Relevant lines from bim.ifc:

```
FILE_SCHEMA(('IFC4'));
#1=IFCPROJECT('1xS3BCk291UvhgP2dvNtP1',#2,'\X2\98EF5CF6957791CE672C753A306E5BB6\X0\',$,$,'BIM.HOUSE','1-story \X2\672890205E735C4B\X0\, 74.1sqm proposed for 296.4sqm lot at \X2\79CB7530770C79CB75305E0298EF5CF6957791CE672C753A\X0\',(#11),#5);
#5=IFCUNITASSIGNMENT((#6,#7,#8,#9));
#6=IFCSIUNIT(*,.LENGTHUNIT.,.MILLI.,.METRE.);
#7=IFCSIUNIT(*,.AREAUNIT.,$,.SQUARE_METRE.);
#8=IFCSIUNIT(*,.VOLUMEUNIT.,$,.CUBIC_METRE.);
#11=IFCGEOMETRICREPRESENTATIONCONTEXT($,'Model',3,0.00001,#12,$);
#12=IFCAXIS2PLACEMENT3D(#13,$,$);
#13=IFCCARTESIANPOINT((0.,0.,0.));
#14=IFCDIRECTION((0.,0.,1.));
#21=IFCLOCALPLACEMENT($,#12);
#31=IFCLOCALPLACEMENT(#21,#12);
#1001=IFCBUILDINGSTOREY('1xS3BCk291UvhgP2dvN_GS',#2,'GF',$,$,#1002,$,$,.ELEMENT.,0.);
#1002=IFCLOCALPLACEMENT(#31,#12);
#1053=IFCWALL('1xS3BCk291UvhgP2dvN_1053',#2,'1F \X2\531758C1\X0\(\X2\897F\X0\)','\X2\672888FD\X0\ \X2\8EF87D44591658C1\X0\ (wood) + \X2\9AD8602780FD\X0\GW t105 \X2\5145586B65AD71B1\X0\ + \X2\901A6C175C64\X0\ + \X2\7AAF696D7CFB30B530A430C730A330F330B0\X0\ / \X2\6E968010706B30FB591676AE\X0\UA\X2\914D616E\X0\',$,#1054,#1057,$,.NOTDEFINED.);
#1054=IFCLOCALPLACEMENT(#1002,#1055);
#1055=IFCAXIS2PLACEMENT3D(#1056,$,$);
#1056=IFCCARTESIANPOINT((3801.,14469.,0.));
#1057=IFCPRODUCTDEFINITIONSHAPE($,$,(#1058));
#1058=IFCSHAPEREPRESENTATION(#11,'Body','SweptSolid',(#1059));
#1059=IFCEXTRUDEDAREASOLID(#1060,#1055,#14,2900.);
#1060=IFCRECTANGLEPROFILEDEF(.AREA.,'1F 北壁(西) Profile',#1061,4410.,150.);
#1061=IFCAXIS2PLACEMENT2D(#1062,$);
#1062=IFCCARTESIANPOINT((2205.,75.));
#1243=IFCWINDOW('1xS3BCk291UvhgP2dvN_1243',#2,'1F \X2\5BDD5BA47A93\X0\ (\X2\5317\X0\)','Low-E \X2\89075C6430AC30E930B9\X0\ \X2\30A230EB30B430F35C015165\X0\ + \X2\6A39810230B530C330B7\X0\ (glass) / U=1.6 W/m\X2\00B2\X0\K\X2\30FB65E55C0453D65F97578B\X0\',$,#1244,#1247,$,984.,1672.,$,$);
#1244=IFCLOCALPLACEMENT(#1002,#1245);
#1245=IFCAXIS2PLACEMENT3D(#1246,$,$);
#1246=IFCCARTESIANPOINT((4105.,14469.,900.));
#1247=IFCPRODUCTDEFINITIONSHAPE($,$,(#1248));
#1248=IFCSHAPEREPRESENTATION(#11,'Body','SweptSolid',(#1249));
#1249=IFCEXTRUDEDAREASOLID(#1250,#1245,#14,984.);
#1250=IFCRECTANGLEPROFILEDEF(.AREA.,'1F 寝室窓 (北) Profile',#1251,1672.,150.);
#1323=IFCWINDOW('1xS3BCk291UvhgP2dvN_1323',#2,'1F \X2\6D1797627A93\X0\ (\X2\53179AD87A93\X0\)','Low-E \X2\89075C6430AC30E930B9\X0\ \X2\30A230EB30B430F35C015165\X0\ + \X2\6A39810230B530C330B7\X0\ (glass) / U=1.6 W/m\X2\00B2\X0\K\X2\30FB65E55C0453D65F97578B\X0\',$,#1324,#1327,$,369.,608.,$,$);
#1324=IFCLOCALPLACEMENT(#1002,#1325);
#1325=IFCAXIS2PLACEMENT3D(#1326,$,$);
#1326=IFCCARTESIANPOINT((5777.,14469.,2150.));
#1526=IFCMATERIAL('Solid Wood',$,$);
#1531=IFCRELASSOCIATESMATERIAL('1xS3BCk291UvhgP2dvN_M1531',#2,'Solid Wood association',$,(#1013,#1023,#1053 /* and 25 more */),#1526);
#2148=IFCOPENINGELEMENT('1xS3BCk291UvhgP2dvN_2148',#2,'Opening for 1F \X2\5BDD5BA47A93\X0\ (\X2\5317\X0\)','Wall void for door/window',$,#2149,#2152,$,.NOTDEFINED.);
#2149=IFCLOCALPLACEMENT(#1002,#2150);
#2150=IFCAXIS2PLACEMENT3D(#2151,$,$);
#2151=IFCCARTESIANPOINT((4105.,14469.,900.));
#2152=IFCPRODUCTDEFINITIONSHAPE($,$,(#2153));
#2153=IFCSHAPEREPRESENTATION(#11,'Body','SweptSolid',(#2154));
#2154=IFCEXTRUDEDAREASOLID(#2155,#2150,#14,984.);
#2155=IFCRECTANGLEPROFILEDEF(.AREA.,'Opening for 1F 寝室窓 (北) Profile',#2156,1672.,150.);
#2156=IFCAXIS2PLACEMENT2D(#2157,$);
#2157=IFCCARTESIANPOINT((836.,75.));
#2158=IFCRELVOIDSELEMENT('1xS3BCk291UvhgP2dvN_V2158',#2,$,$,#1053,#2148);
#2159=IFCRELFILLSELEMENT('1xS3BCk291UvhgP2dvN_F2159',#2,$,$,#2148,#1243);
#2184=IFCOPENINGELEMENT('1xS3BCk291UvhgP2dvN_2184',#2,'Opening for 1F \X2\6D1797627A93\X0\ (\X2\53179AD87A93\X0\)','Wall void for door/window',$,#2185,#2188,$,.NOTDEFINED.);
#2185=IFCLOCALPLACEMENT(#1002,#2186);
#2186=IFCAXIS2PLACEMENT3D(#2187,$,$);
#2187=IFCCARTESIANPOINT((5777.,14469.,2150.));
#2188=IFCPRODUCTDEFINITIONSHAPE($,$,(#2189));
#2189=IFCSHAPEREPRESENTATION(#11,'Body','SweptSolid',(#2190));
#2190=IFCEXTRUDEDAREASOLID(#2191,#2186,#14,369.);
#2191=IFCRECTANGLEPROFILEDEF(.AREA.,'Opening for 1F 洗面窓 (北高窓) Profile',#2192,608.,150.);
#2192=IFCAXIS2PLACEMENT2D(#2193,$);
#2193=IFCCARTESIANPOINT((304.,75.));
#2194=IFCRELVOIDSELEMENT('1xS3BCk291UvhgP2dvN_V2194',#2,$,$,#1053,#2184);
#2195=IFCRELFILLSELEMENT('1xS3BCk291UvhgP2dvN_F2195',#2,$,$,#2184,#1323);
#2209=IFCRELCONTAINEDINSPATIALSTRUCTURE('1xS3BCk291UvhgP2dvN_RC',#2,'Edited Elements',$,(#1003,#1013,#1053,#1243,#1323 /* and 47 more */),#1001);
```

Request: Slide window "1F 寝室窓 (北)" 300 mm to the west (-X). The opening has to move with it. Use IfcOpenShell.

```python
import ifcopenshell
import ifcopenshell.api.geometry
import ifcopenshell.util.placement

model = ifcopenshell.open("bim.ifc")

window = model.by_guid("1xS3BCk291UvhgP2dvN_1243")
opening = window.FillsVoids[0].RelatingOpeningElement
wall = opening.VoidsElements[0].RelatingBuildingElement

wall_matrix = ifcopenshell.util.placement.get_local_placement(wall.ObjectPlacement)
shift = wall_matrix[:3, 0] * -300.0
before = ifcopenshell.util.placement.get_local_placement(window.ObjectPlacement)[:3, 3].copy()

# The window is not placed relative to its opening, so move both.
for product in (opening, window):
    matrix = ifcopenshell.util.placement.get_local_placement(product.ObjectPlacement)
    matrix[:3, 3] += shift
    ifcopenshell.api.geometry.edit_object_placement(model, product=product, matrix=matrix, is_si=False)

after = ifcopenshell.util.placement.get_local_placement(window.ObjectPlacement)[:3, 3]
print("window moved by", (after - before).round(3) + 0.0)

model.write("bim-out.ifc")
```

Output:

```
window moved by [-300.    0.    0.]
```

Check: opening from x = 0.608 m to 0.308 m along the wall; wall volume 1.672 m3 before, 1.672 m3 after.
